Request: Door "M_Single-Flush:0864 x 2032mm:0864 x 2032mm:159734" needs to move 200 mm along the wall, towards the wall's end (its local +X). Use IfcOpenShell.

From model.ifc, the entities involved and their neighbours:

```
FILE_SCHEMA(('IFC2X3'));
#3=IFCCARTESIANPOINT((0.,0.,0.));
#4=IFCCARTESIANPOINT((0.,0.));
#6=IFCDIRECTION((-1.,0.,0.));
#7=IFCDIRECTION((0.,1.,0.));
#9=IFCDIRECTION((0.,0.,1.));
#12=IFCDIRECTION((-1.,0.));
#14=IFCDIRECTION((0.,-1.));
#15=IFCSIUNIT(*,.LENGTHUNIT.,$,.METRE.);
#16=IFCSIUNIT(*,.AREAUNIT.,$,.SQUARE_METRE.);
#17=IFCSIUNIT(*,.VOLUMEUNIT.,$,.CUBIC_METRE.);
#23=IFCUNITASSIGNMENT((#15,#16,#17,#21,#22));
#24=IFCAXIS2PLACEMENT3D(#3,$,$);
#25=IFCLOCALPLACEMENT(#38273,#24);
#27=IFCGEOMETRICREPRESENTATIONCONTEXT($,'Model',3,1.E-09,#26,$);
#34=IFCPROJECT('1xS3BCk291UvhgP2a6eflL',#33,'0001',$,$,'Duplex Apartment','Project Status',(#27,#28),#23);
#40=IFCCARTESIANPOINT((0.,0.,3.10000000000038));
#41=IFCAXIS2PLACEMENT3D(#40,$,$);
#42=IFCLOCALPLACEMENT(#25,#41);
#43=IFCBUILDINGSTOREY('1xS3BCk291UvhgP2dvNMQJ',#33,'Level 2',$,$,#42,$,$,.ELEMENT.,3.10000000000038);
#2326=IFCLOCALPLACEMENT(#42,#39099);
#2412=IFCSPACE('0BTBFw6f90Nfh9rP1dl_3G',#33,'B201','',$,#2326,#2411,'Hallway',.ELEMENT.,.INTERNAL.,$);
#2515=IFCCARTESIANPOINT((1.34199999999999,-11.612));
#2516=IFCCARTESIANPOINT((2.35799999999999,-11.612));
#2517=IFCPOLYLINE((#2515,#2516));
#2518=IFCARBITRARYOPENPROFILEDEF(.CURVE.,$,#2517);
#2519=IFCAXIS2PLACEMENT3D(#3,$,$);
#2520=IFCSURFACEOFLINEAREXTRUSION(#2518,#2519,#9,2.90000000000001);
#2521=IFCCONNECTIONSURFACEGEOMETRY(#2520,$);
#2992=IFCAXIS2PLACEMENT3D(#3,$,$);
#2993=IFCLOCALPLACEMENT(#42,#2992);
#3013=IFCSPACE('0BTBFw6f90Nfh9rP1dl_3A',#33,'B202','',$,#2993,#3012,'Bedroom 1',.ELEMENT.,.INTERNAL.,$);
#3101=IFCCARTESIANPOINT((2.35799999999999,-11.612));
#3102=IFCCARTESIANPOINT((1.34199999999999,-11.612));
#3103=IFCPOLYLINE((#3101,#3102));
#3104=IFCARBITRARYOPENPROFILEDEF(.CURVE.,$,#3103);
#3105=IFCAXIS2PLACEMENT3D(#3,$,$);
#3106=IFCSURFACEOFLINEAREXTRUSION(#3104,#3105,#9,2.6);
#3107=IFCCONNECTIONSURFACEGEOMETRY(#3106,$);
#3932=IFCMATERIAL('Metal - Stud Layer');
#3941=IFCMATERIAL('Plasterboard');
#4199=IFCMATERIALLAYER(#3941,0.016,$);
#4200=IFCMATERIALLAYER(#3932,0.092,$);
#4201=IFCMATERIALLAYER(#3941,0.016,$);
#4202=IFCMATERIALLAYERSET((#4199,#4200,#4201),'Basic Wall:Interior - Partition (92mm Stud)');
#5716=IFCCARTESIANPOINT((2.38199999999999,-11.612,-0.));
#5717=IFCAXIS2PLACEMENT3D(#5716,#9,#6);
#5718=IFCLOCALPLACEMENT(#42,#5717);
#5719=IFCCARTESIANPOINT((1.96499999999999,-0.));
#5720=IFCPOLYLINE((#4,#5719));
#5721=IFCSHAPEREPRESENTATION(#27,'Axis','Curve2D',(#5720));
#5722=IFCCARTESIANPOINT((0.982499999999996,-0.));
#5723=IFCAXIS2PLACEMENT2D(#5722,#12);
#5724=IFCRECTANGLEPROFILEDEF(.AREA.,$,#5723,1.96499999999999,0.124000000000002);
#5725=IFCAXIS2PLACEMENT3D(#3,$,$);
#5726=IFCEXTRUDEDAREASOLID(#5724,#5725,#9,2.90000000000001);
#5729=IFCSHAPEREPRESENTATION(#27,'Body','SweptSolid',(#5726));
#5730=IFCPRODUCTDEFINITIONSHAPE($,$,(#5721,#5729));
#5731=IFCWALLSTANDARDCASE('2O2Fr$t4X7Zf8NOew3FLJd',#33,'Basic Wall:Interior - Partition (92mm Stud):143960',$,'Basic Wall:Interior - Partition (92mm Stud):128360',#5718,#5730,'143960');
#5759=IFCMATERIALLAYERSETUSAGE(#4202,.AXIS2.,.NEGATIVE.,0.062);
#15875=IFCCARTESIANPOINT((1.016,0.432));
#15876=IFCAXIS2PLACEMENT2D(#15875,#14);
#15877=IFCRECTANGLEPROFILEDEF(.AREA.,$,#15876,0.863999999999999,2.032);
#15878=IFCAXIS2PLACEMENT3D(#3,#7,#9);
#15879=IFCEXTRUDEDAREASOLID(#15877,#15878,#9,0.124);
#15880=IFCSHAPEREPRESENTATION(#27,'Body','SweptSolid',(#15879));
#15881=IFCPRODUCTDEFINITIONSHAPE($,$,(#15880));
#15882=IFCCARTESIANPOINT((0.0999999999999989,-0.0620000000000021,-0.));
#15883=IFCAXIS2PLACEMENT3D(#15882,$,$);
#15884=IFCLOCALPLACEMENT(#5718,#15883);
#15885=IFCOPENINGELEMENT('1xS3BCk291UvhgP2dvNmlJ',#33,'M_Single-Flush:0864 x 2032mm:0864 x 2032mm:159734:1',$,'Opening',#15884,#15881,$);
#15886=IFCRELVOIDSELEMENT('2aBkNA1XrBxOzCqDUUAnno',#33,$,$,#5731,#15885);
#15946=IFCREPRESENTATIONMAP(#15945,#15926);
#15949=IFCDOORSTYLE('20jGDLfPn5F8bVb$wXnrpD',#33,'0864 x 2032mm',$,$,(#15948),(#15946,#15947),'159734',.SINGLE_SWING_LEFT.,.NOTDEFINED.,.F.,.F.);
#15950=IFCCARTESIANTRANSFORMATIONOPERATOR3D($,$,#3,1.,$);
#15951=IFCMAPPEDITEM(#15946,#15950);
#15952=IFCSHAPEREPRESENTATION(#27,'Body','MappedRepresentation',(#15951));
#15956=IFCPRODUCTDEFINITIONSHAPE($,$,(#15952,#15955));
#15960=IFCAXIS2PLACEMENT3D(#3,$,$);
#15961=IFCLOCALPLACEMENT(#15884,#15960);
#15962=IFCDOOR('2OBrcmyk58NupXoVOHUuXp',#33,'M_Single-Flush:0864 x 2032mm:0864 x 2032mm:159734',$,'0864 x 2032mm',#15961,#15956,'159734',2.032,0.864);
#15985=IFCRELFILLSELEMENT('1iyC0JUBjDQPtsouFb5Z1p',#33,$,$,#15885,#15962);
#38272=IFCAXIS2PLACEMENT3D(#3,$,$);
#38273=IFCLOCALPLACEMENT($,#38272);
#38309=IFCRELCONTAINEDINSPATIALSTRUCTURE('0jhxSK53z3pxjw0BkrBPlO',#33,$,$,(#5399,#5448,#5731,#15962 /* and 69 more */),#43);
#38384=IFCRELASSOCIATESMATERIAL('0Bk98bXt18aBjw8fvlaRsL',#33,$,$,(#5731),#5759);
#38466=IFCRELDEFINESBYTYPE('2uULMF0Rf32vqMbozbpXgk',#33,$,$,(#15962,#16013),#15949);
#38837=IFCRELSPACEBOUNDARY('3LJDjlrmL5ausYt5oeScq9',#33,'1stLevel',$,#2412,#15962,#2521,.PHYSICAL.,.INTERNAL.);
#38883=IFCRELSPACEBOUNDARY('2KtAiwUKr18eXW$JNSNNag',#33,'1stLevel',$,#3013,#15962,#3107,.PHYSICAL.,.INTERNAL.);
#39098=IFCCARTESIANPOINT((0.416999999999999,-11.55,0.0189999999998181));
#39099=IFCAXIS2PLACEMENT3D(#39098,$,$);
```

```python
import numpy as np
import ifcopenshell
import ifcopenshell.api.geometry
import ifcopenshell.util.placement
import ifcopenshell.util.unit

model = ifcopenshell.open("model.ifc")
unit_scale = ifcopenshell.util.unit.calculate_unit_scale(model)

door = model.by_guid("2OBrcmyk58NupXoVOHUuXp")
opening = door.FillsVoids[0].RelatingOpeningElement
wall = opening.VoidsElements[0].RelatingBuildingElement

wall_matrix = ifcopenshell.util.placement.get_local_placement(wall.ObjectPlacement)
shift = wall_matrix[:3, 0] * 0.2 / unit_scale
before = ifcopenshell.util.placement.get_local_placement(door.ObjectPlacement)[:3, 3].copy()

# The door is placed relative to its opening, so it follows when the opening moves.
matrix = ifcopenshell.util.placement.get_local_placement(opening.ObjectPlacement)
matrix[:3, 3] += shift
ifcopenshell.api.geometry.edit_object_placement(
    model, product=opening, matrix=matrix, is_si=False, should_transform_children=True
)

# Space boundary surfaces are stored in each space's coordinates; move them too.
for rel in door.ProvidesBoundaries:
    if not rel.ConnectionGeometry:
        continue
    surface = rel.ConnectionGeometry.SurfaceOnRelatingElement
    space_matrix = ifcopenshell.util.placement.get_local_placement(rel.RelatingSpace.ObjectPlacement)
    point = np.array(surface.Position.Location.Coordinates) + space_matrix[:3, :3].T @ shift
    surface.Position = model.createIfcAxis2Placement3D(
        model.createIfcCartesianPoint(point.tolist()), surface.Position.Axis, surface.Position.RefDirection
    )

after = ifcopenshell.util.placement.get_local_placement(door.ObjectPlacement)[:3, 3]
print("door moved by", (after - before).round(3) + 0.0)

model.write("model_rev.ifc")
```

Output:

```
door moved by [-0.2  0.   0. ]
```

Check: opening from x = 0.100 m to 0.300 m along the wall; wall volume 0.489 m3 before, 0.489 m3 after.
